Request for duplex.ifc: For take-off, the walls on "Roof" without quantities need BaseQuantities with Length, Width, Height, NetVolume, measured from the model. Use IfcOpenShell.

First a look at what the model holds.

```python
import ifcopenshell
import ifcopenshell.util.element
import ifcopenshell.util.unit

model = ifcopenshell.open("duplex.ifc")
print(model.schema)
for unit_type in ("LENGTHUNIT", "AREAUNIT", "VOLUMEUNIT"):
    print(unit_type, ifcopenshell.util.unit.calculate_unit_scale(model, unit_type))
storey = next(s for s in model.by_type("IfcBuildingStorey") if s.Name == "Roof")
walls = [e for e in ifcopenshell.util.element.get_decomposition(storey) if e.is_a("IfcWall")]
for e in sorted(walls, key=lambda e: e.id()):
    print(e.id(), e.is_a(), e.Name, list(ifcopenshell.util.element.get_psets(e, qtos_only=True)), sep=" | ")
```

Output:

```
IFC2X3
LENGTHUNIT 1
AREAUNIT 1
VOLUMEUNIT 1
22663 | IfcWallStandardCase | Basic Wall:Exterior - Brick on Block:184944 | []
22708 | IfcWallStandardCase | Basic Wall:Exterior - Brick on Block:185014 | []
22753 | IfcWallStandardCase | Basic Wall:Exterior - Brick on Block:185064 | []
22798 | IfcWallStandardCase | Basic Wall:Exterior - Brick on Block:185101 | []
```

```python
import ifcopenshell
import ifcopenshell.api.pset
import ifcopenshell.geom
import ifcopenshell.util.element
import ifcopenshell.util.shape
import ifcopenshell.util.unit

model = ifcopenshell.open("duplex.ifc")
unit_scale = ifcopenshell.util.unit.calculate_unit_scale(model)
volume_scale = ifcopenshell.util.unit.calculate_unit_scale(model, "VOLUMEUNIT")
settings = ifcopenshell.geom.settings()

storey = next(s for s in model.by_type("IfcBuildingStorey") if s.Name == "Roof")
walls = [e for e in ifcopenshell.util.element.get_decomposition(storey) if e.is_a("IfcWall")]

for e in sorted(walls, key=lambda e: e.id()):
    if ifcopenshell.util.element.get_psets(e, qtos_only=True, should_inherit=False):
        continue
    # Geometry comes back in metres, in the element's own axes.
    shape = ifcopenshell.geom.create_shape(settings, e)
    values = {
        "Length": ifcopenshell.util.shape.get_x(shape.geometry) / unit_scale,
        "Width": ifcopenshell.util.shape.get_y(shape.geometry) / unit_scale,
        "Height": ifcopenshell.util.shape.get_z(shape.geometry) / unit_scale,
        "NetVolume": ifcopenshell.util.shape.get_volume(shape.geometry) / volume_scale,
    }
    qto = ifcopenshell.api.pset.add_qto(model, product=e, name="BaseQuantities")
    ifcopenshell.api.pset.edit_qto(model, qto=qto, properties=values)
    print(e.id(), {k: round(v, 3) for k, v in values.items()})

model.write("duplex_updated.ifc")
```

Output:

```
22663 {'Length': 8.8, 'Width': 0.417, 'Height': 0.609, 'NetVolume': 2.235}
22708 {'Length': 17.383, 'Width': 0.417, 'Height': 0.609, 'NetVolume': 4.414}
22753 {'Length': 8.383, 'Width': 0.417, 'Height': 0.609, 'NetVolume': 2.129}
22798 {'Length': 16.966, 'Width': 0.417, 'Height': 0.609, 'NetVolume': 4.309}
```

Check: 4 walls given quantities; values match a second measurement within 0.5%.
